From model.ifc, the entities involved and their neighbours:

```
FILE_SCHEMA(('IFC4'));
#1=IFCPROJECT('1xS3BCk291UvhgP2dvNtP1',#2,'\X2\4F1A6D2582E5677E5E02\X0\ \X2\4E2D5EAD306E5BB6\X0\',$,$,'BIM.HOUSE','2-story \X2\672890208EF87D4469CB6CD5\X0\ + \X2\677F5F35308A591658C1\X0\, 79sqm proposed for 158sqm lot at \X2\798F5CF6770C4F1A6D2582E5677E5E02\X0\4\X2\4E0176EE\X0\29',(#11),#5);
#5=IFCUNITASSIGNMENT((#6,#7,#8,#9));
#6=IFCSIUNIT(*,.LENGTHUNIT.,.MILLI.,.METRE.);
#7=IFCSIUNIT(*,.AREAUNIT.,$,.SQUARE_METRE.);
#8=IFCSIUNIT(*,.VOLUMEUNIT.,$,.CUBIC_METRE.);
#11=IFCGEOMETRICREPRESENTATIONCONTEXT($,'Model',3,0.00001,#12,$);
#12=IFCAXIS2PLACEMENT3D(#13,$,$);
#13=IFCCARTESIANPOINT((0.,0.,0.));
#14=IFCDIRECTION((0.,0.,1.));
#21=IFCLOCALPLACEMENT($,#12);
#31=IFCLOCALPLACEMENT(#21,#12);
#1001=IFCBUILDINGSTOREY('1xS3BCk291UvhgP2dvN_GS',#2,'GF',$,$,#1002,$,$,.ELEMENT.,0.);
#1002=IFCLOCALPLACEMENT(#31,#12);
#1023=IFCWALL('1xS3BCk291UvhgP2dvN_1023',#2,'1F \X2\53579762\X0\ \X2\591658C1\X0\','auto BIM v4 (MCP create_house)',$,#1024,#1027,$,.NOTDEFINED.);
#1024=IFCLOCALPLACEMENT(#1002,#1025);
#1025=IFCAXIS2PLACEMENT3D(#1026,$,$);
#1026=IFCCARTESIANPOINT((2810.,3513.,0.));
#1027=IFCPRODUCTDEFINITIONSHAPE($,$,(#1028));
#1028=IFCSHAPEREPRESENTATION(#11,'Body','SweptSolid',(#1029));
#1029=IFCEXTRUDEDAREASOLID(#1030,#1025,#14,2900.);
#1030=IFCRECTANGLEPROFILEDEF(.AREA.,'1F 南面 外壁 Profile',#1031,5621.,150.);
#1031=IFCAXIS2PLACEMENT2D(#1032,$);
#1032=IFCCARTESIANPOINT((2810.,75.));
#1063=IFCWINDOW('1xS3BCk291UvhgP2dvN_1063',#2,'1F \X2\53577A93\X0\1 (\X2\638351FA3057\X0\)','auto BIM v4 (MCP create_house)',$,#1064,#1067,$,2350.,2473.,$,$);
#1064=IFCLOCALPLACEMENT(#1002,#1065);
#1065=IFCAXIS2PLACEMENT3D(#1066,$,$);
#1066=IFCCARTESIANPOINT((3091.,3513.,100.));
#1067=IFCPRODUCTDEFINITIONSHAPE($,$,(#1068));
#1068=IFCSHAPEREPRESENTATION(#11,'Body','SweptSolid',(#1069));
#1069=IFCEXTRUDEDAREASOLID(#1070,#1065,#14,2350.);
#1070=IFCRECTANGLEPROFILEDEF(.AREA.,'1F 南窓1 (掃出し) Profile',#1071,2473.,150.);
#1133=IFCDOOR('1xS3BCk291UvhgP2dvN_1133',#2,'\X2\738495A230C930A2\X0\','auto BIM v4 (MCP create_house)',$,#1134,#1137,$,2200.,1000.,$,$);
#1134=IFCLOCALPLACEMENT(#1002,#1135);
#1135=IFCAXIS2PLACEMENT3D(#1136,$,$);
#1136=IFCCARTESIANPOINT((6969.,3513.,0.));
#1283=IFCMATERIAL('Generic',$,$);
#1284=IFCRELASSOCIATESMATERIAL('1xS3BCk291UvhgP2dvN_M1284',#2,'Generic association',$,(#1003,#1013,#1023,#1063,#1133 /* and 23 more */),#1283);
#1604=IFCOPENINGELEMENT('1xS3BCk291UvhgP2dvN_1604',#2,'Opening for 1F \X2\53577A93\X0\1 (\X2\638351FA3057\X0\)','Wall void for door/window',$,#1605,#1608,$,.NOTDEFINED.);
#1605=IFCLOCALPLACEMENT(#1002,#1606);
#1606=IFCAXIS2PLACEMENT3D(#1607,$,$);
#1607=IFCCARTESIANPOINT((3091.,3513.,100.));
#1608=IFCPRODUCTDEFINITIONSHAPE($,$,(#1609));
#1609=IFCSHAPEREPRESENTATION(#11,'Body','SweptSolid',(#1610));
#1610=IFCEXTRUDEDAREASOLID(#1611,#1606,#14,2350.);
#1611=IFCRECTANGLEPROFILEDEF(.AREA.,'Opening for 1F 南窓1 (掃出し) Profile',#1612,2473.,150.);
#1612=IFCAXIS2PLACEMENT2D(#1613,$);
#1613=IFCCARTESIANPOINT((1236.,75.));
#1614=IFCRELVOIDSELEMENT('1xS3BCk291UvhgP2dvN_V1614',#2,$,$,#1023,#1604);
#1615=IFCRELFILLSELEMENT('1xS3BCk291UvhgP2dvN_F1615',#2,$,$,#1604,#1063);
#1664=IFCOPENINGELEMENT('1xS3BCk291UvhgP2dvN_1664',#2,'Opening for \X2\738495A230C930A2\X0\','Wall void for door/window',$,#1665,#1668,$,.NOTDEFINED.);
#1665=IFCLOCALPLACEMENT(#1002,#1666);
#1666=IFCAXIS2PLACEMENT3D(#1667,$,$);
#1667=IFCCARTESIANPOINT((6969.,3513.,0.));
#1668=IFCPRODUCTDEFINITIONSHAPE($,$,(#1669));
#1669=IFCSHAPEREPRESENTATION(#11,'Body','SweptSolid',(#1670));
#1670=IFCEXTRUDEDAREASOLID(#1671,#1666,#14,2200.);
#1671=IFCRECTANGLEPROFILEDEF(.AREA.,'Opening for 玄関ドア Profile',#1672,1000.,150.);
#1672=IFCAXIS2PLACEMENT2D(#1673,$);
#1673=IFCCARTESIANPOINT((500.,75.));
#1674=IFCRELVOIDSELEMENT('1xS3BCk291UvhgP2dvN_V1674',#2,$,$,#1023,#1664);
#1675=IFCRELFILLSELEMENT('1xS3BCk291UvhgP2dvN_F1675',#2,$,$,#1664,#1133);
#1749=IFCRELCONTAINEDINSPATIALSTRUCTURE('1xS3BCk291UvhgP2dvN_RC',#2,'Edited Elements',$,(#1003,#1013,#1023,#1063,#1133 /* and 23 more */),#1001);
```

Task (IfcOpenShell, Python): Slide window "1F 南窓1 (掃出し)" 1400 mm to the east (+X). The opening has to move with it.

```python
import ifcopenshell
import ifcopenshell.api.geometry
import ifcopenshell.util.placement

model = ifcopenshell.open("model.ifc")

window = model.by_id(1063)
opening = window.FillsVoids[0].RelatingOpeningElement
wall = opening.VoidsElements[0].RelatingBuildingElement

wall_matrix = ifcopenshell.util.placement.get_local_placement(wall.ObjectPlacement)
shift = wall_matrix[:3, 0] * 1400.0
before = ifcopenshell.util.placement.get_local_placement(window.ObjectPlacement)[:3, 3].copy()

# The window is not placed relative to its opening, so move both.
for product in (opening, window):
    matrix = ifcopenshell.util.placement.get_local_placement(product.ObjectPlacement)
    matrix[:3, 3] += shift
    ifcopenshell.api.geometry.edit_object_placement(model, product=product, matrix=matrix, is_si=False)

after = ifcopenshell.util.placement.get_local_placement(window.ObjectPlacement)[:3, 3]
print("window moved by", (after - before).round(3) + 0.0)

model.write("model_updated.ifc")
```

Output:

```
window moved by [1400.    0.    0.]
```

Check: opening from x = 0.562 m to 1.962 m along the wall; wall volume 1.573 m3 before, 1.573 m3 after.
